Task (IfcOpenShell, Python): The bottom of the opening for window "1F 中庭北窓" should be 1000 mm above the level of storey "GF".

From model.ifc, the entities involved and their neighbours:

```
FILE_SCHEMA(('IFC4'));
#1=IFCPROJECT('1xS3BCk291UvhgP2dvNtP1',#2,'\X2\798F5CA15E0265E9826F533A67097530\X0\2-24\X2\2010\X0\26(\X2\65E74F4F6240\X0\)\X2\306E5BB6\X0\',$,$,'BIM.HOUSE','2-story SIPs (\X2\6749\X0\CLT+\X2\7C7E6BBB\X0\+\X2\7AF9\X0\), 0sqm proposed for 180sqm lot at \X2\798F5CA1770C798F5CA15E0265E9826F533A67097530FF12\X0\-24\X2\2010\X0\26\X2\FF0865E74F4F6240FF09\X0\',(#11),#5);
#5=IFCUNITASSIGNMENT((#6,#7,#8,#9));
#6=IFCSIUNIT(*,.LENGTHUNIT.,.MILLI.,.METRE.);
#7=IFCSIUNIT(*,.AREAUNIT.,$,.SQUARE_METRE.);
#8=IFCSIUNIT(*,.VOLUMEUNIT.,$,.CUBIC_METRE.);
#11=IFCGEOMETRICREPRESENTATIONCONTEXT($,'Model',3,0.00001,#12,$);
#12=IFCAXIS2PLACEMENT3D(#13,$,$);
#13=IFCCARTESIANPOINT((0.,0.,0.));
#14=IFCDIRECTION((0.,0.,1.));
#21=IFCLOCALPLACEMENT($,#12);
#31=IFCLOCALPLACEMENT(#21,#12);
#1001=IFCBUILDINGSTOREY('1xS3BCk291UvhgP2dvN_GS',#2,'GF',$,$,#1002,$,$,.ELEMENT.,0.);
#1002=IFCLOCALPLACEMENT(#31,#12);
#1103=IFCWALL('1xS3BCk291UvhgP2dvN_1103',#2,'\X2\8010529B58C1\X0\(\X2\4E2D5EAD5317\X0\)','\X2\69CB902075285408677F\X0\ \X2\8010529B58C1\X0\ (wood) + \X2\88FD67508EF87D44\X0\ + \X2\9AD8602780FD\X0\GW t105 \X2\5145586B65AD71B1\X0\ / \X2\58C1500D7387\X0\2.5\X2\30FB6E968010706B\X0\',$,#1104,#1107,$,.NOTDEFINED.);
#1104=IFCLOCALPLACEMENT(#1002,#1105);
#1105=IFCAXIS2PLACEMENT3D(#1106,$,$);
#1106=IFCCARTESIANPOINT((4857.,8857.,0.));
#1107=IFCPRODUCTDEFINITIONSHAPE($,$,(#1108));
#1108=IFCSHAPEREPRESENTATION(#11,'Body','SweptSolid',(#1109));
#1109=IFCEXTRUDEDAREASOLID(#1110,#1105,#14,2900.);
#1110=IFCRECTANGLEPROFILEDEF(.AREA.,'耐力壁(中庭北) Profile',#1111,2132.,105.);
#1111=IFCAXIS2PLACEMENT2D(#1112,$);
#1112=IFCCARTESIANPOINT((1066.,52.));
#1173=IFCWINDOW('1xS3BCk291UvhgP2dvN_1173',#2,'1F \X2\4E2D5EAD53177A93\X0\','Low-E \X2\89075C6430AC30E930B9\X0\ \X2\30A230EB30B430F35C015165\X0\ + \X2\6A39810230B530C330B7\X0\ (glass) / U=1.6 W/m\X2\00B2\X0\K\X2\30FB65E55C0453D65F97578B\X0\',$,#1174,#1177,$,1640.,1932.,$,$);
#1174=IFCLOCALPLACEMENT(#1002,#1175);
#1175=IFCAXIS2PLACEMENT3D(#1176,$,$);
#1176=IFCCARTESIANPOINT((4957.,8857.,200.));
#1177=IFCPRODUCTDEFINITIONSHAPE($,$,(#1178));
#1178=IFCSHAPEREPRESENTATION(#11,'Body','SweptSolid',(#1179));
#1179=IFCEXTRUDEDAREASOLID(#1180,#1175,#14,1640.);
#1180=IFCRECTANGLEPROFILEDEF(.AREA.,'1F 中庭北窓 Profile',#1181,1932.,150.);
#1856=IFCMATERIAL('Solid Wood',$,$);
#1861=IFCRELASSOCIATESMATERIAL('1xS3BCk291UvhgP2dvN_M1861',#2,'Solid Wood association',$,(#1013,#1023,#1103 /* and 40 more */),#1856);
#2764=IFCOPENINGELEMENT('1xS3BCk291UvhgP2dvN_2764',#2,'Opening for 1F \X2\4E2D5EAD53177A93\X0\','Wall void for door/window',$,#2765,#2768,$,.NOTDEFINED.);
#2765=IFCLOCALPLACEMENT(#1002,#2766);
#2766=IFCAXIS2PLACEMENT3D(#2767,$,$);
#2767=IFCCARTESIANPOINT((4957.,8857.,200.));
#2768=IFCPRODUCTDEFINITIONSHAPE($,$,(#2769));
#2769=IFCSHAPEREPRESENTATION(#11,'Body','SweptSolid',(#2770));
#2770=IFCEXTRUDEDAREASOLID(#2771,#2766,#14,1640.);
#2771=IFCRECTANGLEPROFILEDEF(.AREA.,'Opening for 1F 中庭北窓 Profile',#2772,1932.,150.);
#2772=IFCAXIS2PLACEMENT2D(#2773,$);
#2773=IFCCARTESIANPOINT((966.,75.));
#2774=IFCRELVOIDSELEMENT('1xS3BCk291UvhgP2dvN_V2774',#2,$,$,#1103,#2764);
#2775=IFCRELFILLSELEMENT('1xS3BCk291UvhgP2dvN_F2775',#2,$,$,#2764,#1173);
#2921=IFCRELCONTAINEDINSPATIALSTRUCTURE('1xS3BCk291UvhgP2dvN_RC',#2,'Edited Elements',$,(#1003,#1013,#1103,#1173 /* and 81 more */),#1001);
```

```python
import numpy as np
import ifcopenshell
import ifcopenshell.api.geometry
import ifcopenshell.geom
import ifcopenshell.util.element
import ifcopenshell.util.placement
import ifcopenshell.util.shape
import ifcopenshell.util.unit

model = ifcopenshell.open("model.ifc")
unit_scale = ifcopenshell.util.unit.calculate_unit_scale(model)

window = model.by_id(1173)
opening = window.FillsVoids[0].RelatingOpeningElement
storey = ifcopenshell.util.element.get_container(window, ifc_class="IfcBuildingStorey")
level = ifcopenshell.util.placement.get_local_placement(storey.ObjectPlacement)[2, 3]

# The opening's origin need not be at the sill, so measure its lowest point.
shape = ifcopenshell.geom.create_shape(ifcopenshell.geom.settings(), opening)
bottom = ifcopenshell.util.shape.get_shape_bottom_elevation(shape, shape.geometry) / unit_scale
dz = level + 1 / unit_scale - bottom

shift = np.array([0.0, 0.0, dz])
# The window is not placed relative to its opening, so move both.
for product in (opening, window):
    matrix = ifcopenshell.util.placement.get_local_placement(product.ObjectPlacement)
    matrix[:3, 3] += shift
    ifcopenshell.api.geometry.edit_object_placement(model, product=product, matrix=matrix, is_si=False)

print(f"moved by {dz * unit_scale:+.3f} m")

model.write("model_edited.ifc")
```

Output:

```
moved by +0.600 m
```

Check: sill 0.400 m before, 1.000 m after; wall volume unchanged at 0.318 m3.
